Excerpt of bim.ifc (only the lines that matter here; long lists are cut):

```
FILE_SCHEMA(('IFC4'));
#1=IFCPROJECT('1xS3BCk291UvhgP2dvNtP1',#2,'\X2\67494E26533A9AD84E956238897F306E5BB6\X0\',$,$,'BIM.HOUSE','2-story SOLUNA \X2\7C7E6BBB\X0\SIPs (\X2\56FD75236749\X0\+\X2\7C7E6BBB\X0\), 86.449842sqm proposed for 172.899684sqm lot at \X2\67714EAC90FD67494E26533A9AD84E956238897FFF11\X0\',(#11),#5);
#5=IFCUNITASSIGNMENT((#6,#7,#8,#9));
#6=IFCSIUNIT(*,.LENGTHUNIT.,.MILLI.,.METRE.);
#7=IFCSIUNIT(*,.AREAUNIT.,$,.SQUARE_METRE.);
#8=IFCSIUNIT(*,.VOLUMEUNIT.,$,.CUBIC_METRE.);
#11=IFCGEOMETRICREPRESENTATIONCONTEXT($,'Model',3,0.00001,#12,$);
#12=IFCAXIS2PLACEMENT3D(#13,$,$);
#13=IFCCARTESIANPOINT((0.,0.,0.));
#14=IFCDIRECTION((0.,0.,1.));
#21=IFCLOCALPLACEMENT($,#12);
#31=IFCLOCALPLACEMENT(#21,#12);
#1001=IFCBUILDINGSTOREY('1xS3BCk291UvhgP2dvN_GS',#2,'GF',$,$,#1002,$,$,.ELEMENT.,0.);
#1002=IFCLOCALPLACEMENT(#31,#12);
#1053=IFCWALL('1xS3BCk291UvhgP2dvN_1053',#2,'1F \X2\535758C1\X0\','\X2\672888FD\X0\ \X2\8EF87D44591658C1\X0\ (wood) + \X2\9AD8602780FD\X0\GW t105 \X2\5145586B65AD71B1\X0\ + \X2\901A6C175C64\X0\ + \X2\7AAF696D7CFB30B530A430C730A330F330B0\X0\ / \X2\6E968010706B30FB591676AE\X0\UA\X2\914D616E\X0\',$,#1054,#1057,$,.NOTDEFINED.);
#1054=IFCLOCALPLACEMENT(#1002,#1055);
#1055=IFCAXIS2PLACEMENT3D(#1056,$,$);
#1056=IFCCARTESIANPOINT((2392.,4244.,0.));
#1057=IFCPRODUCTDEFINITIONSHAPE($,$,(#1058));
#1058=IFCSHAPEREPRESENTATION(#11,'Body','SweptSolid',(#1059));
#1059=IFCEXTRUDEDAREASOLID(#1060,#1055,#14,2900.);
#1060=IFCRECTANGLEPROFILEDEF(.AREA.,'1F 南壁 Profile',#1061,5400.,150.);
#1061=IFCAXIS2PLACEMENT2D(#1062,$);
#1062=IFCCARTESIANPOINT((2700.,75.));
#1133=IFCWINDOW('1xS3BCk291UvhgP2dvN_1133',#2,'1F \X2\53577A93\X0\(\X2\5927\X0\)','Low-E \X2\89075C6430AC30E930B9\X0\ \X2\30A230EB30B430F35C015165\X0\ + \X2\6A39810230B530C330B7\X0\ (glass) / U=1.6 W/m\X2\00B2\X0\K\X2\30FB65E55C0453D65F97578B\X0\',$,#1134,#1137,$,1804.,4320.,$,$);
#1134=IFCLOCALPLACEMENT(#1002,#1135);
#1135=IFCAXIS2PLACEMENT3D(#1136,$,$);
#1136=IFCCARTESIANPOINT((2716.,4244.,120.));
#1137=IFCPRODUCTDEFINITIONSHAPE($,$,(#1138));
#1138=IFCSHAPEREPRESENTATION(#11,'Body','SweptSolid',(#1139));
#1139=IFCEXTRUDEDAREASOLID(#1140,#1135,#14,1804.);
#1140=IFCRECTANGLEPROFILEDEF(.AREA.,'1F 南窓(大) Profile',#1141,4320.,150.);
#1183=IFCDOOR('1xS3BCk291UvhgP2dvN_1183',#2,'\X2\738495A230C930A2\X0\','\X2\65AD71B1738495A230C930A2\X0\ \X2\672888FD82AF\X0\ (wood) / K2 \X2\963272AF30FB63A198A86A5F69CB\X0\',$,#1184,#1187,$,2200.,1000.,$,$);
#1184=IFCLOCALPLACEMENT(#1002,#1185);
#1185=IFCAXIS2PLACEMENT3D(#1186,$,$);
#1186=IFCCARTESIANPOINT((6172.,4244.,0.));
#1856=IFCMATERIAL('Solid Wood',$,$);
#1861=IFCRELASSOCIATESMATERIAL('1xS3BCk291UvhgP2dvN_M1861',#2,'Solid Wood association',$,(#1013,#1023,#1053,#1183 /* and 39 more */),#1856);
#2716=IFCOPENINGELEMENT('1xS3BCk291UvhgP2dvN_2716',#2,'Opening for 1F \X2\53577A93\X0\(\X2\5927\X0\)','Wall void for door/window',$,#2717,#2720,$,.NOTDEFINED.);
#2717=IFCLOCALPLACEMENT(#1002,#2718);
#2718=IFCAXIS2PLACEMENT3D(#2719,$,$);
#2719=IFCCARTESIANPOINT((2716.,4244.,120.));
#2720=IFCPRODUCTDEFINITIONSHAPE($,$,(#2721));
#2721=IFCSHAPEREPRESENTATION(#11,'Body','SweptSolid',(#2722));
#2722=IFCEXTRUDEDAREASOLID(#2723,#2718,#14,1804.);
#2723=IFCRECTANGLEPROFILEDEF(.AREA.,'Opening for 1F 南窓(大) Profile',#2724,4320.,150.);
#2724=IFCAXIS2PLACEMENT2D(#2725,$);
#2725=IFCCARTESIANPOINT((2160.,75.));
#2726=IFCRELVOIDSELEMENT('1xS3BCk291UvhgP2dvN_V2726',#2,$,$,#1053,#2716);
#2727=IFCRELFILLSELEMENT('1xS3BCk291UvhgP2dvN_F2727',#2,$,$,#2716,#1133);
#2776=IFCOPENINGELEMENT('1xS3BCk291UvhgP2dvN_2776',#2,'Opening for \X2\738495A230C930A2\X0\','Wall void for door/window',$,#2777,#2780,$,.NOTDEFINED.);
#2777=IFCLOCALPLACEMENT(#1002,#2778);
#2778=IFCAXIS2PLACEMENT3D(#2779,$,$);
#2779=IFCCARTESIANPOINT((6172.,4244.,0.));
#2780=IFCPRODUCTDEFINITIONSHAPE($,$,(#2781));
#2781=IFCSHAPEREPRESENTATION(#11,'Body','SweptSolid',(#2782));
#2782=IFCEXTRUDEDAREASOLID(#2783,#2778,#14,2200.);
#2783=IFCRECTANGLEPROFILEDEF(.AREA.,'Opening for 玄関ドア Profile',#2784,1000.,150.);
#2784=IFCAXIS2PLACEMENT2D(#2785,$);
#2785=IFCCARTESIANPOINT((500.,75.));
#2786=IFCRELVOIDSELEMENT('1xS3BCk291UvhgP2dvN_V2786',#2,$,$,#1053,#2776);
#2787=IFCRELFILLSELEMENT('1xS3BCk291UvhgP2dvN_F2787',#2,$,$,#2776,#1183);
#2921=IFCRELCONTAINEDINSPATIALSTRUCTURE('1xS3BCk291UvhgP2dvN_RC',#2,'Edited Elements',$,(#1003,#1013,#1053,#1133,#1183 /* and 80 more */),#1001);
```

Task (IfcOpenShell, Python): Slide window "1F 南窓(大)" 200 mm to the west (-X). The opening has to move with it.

```python
import ifcopenshell
import ifcopenshell.api.geometry
import ifcopenshell.util.placement

model = ifcopenshell.open("bim.ifc")

window = model.by_id(1133)
opening = window.FillsVoids[0].RelatingOpeningElement
wall = opening.VoidsElements[0].RelatingBuildingElement

wall_matrix = ifcopenshell.util.placement.get_local_placement(wall.ObjectPlacement)
shift = wall_matrix[:3, 0] * -200.0
before = ifcopenshell.util.placement.get_local_placement(window.ObjectPlacement)[:3, 3].copy()

# The window is not placed relative to its opening, so move both.
for product in (opening, window):
    matrix = ifcopenshell.util.placement.get_local_placement(product.ObjectPlacement)
    matrix[:3, 3] += shift
    ifcopenshell.api.geometry.edit_object_placement(model, product=product, matrix=matrix, is_si=False)

after = ifcopenshell.util.placement.get_local_placement(window.ObjectPlacement)[:3, 3]
print("window moved by", (after - before).round(3) + 0.0)

model.write("bim-out.ifc")
```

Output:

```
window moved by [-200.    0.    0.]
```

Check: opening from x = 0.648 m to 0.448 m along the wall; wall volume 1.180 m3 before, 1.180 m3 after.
